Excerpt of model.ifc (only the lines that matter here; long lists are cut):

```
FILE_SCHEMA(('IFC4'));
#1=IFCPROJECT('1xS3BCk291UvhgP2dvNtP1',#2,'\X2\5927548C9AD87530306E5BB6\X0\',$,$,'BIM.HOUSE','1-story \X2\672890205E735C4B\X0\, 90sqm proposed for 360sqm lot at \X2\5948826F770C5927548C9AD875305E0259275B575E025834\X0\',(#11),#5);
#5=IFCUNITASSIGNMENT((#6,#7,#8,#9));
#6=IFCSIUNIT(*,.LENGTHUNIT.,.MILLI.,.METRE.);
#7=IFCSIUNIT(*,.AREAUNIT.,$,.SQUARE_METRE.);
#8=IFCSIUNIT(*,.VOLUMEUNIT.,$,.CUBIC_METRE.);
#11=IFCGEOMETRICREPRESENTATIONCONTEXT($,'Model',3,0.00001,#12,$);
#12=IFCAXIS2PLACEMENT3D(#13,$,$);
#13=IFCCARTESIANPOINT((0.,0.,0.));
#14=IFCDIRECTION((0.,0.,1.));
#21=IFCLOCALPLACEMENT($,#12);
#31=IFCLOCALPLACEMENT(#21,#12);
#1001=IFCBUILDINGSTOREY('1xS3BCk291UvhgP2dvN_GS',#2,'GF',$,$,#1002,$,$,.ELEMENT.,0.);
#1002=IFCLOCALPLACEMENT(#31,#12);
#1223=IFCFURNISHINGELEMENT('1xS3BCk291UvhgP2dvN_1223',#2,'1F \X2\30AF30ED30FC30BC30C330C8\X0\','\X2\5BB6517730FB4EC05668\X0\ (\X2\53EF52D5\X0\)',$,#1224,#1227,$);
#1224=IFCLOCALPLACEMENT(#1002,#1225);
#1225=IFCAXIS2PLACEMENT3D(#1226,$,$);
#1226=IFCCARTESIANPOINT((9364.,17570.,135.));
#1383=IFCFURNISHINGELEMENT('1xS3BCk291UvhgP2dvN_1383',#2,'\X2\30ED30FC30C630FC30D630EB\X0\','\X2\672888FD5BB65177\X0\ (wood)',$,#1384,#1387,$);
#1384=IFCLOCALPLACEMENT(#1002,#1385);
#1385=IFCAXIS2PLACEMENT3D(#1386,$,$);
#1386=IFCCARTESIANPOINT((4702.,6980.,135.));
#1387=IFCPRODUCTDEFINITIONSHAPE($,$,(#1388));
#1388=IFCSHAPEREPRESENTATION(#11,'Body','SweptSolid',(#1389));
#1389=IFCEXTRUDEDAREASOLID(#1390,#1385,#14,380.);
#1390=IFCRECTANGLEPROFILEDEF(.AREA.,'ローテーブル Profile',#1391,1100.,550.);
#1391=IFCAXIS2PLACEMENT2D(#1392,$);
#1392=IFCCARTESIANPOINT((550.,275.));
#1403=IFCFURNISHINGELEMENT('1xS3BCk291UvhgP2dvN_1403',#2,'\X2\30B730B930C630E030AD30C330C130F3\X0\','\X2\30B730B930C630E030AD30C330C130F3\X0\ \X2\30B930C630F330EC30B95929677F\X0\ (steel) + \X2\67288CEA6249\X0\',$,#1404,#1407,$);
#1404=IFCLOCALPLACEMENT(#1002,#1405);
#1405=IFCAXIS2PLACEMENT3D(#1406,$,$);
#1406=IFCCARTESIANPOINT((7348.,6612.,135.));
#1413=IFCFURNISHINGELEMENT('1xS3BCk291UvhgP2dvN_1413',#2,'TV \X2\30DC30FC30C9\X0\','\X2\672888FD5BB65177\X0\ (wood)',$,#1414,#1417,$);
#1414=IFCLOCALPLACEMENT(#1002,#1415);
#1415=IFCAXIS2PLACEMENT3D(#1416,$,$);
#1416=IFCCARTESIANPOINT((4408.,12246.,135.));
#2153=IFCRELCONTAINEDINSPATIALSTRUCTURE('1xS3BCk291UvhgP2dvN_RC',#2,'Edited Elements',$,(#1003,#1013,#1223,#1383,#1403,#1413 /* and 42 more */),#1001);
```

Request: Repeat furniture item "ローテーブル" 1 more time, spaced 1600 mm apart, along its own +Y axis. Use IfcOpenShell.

```python
import ifcopenshell
import ifcopenshell.api.geometry
import ifcopenshell.api.root
import ifcopenshell.util.element
import ifcopenshell.util.placement

model = ifcopenshell.open("model.ifc")


def reuse_history(source, copy):
    """copy_class also copies each property set's owner history, people and application; keep the originals."""
    for rel in copy.IsDefinedBy:
        if rel.is_a("IfcRelDefinesByProperties") and (history := rel.RelatingPropertyDefinition.OwnerHistory):
            rel.RelatingPropertyDefinition.OwnerHistory = source.OwnerHistory
            ifcopenshell.util.element.remove_deep2(model, history)


source = model.by_guid("1xS3BCk291UvhgP2dvN_1383")
base = ifcopenshell.util.placement.get_local_placement(source.ObjectPlacement)
step = base[:3, 1] * 1600.0

for i in range(1, 2):
    copy = ifcopenshell.api.root.copy_class(model, product=source)
    copy.Representation = ifcopenshell.util.element.copy_deep(
        model, source.Representation, exclude=["IfcGeometricRepresentationContext", "IfcRepresentationMap"]
    )
    reuse_history(source, copy)
    matrix = base.copy()
    matrix[:3, 3] += i * step
    print("added at", matrix[:3, 3].round(3) + 0.0)
    ifcopenshell.api.geometry.edit_object_placement(model, product=copy, matrix=matrix, is_si=False)

model.write("model_updated.ifc")
```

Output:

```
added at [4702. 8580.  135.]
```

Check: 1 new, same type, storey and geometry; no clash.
